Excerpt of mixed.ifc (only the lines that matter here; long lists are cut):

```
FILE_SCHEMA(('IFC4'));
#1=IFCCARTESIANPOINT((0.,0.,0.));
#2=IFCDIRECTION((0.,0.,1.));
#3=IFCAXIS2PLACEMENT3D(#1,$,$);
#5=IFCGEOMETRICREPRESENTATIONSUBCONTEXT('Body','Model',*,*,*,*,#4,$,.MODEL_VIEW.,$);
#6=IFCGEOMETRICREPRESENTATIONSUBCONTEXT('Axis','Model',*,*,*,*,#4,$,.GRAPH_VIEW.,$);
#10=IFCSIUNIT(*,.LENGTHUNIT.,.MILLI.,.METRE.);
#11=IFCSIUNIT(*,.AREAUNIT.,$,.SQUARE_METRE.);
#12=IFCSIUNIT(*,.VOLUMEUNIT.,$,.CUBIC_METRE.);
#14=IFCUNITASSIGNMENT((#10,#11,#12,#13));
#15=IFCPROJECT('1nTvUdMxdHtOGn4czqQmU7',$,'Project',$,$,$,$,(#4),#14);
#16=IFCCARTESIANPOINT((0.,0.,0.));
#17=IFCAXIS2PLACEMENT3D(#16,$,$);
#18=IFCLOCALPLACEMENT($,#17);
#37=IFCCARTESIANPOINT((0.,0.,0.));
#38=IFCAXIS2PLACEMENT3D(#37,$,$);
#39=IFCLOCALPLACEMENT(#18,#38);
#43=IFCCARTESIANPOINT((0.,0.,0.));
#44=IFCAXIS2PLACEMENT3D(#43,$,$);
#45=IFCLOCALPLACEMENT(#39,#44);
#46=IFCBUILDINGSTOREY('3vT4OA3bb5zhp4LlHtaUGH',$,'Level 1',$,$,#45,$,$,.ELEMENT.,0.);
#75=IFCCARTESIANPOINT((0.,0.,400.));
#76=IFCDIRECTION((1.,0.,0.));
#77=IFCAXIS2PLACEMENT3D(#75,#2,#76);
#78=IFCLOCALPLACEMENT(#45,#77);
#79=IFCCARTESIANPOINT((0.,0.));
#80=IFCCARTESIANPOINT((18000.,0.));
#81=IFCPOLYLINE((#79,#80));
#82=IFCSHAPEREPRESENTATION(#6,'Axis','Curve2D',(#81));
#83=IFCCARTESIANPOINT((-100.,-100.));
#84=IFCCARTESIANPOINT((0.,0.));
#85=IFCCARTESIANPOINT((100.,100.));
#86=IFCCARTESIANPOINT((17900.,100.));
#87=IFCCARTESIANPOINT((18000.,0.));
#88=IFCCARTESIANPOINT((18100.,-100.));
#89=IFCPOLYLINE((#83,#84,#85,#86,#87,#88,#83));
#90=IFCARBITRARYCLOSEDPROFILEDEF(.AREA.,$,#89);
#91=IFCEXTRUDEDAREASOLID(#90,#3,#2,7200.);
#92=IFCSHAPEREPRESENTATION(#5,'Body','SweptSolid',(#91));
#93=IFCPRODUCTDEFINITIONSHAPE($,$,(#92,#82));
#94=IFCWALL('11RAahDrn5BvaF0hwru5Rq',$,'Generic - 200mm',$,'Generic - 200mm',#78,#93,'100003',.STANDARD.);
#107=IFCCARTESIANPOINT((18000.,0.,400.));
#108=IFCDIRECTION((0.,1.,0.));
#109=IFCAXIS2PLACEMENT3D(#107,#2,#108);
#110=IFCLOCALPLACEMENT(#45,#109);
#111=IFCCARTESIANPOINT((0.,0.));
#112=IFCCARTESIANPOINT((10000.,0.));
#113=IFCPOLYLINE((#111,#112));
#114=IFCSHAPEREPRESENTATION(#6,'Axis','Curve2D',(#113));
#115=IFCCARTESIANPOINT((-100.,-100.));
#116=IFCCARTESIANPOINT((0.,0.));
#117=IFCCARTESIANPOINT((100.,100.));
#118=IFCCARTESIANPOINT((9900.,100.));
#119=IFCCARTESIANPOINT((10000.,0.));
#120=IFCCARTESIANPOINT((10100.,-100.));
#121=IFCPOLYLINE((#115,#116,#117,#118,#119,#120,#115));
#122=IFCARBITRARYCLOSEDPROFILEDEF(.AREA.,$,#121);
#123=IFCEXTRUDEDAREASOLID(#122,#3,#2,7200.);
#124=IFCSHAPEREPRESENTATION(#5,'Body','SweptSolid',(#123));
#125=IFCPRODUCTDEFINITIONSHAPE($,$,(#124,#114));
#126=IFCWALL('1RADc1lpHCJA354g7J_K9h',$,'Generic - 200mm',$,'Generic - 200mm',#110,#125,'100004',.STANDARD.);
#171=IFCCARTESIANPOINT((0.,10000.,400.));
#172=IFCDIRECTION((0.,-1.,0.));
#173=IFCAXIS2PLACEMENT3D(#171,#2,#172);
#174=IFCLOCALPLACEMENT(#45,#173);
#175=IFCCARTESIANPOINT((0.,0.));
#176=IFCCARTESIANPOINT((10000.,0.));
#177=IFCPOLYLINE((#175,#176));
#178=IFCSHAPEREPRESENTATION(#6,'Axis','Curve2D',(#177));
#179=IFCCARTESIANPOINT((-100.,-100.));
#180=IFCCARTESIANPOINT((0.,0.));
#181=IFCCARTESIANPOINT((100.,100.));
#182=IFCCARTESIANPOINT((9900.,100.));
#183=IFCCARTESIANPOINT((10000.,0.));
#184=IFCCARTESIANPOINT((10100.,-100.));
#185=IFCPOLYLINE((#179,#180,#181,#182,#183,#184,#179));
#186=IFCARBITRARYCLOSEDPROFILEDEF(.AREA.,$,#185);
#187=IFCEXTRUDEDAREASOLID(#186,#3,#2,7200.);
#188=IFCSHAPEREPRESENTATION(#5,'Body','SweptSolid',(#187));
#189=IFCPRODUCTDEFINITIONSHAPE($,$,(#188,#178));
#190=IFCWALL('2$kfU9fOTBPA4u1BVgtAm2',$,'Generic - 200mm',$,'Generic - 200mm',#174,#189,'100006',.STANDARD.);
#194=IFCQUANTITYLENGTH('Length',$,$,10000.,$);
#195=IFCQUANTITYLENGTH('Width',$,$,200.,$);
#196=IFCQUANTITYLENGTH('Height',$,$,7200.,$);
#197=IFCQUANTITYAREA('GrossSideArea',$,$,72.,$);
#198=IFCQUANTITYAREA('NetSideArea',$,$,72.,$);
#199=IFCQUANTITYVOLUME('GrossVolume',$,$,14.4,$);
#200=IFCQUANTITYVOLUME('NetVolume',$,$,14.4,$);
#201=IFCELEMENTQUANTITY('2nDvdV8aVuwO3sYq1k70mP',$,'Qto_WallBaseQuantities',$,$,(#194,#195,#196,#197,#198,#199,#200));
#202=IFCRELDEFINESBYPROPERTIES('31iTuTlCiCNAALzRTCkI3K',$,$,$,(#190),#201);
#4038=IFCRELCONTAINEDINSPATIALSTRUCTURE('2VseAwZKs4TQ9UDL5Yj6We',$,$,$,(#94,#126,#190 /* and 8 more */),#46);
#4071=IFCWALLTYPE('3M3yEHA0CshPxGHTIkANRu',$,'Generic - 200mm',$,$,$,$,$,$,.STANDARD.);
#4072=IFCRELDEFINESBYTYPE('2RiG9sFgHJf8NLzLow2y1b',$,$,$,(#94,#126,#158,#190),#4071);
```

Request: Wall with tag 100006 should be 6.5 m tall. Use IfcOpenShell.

```python
import ifcopenshell
import ifcopenshell.api.pset
import ifcopenshell.geom
import ifcopenshell.util.element
import ifcopenshell.util.representation
import ifcopenshell.util.shape
import ifcopenshell.util.unit

model = ifcopenshell.open("mixed.ifc")
unit_scale = ifcopenshell.util.unit.calculate_unit_scale(model)
area_scale = ifcopenshell.util.unit.calculate_unit_scale(model, "AREAUNIT")
volume_scale = ifcopenshell.util.unit.calculate_unit_scale(model, "VOLUMEUNIT")
settings = ifcopenshell.geom.settings()


def volume(element):
    """Net volume in cubic metres, openings subtracted."""
    shape = ifcopenshell.geom.create_shape(settings, element)
    return ifcopenshell.util.shape.get_volume(shape.geometry)


wall = model.by_id(190)
before = volume(wall)

body = ifcopenshell.util.representation.get_representation(wall, "Model", "Body")
solid = body.Items[0]
old_height = solid.Depth
solid.Depth = 6.5 / unit_scale
after = volume(wall)
thickness = 0.2  # wall thickness in metres

# Update the stored height, areas and volumes.
qto = model.by_id(ifcopenshell.util.element.get_pset(wall, "Qto_WallBaseQuantities", should_inherit=False)["id"])
ifcopenshell.api.pset.edit_qto(model, qto=qto, properties={
    "Height": solid.Depth,
    "GrossSideArea": ifcopenshell.util.element.get_pset(wall, "Qto_WallBaseQuantities", "GrossSideArea") * solid.Depth / old_height,
    "NetSideArea": after / thickness / area_scale,
    "GrossVolume": ifcopenshell.util.element.get_pset(wall, "Qto_WallBaseQuantities", "GrossVolume") * solid.Depth / old_height,
    "NetVolume": after / volume_scale,
})

print(f"height {old_height:g} -> {solid.Depth:g}, volume {before:.3f} -> {after:.3f} m3")

model.write("mixed_rev.ifc")
```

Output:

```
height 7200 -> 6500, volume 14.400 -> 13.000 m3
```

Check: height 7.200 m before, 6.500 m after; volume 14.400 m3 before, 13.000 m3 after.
